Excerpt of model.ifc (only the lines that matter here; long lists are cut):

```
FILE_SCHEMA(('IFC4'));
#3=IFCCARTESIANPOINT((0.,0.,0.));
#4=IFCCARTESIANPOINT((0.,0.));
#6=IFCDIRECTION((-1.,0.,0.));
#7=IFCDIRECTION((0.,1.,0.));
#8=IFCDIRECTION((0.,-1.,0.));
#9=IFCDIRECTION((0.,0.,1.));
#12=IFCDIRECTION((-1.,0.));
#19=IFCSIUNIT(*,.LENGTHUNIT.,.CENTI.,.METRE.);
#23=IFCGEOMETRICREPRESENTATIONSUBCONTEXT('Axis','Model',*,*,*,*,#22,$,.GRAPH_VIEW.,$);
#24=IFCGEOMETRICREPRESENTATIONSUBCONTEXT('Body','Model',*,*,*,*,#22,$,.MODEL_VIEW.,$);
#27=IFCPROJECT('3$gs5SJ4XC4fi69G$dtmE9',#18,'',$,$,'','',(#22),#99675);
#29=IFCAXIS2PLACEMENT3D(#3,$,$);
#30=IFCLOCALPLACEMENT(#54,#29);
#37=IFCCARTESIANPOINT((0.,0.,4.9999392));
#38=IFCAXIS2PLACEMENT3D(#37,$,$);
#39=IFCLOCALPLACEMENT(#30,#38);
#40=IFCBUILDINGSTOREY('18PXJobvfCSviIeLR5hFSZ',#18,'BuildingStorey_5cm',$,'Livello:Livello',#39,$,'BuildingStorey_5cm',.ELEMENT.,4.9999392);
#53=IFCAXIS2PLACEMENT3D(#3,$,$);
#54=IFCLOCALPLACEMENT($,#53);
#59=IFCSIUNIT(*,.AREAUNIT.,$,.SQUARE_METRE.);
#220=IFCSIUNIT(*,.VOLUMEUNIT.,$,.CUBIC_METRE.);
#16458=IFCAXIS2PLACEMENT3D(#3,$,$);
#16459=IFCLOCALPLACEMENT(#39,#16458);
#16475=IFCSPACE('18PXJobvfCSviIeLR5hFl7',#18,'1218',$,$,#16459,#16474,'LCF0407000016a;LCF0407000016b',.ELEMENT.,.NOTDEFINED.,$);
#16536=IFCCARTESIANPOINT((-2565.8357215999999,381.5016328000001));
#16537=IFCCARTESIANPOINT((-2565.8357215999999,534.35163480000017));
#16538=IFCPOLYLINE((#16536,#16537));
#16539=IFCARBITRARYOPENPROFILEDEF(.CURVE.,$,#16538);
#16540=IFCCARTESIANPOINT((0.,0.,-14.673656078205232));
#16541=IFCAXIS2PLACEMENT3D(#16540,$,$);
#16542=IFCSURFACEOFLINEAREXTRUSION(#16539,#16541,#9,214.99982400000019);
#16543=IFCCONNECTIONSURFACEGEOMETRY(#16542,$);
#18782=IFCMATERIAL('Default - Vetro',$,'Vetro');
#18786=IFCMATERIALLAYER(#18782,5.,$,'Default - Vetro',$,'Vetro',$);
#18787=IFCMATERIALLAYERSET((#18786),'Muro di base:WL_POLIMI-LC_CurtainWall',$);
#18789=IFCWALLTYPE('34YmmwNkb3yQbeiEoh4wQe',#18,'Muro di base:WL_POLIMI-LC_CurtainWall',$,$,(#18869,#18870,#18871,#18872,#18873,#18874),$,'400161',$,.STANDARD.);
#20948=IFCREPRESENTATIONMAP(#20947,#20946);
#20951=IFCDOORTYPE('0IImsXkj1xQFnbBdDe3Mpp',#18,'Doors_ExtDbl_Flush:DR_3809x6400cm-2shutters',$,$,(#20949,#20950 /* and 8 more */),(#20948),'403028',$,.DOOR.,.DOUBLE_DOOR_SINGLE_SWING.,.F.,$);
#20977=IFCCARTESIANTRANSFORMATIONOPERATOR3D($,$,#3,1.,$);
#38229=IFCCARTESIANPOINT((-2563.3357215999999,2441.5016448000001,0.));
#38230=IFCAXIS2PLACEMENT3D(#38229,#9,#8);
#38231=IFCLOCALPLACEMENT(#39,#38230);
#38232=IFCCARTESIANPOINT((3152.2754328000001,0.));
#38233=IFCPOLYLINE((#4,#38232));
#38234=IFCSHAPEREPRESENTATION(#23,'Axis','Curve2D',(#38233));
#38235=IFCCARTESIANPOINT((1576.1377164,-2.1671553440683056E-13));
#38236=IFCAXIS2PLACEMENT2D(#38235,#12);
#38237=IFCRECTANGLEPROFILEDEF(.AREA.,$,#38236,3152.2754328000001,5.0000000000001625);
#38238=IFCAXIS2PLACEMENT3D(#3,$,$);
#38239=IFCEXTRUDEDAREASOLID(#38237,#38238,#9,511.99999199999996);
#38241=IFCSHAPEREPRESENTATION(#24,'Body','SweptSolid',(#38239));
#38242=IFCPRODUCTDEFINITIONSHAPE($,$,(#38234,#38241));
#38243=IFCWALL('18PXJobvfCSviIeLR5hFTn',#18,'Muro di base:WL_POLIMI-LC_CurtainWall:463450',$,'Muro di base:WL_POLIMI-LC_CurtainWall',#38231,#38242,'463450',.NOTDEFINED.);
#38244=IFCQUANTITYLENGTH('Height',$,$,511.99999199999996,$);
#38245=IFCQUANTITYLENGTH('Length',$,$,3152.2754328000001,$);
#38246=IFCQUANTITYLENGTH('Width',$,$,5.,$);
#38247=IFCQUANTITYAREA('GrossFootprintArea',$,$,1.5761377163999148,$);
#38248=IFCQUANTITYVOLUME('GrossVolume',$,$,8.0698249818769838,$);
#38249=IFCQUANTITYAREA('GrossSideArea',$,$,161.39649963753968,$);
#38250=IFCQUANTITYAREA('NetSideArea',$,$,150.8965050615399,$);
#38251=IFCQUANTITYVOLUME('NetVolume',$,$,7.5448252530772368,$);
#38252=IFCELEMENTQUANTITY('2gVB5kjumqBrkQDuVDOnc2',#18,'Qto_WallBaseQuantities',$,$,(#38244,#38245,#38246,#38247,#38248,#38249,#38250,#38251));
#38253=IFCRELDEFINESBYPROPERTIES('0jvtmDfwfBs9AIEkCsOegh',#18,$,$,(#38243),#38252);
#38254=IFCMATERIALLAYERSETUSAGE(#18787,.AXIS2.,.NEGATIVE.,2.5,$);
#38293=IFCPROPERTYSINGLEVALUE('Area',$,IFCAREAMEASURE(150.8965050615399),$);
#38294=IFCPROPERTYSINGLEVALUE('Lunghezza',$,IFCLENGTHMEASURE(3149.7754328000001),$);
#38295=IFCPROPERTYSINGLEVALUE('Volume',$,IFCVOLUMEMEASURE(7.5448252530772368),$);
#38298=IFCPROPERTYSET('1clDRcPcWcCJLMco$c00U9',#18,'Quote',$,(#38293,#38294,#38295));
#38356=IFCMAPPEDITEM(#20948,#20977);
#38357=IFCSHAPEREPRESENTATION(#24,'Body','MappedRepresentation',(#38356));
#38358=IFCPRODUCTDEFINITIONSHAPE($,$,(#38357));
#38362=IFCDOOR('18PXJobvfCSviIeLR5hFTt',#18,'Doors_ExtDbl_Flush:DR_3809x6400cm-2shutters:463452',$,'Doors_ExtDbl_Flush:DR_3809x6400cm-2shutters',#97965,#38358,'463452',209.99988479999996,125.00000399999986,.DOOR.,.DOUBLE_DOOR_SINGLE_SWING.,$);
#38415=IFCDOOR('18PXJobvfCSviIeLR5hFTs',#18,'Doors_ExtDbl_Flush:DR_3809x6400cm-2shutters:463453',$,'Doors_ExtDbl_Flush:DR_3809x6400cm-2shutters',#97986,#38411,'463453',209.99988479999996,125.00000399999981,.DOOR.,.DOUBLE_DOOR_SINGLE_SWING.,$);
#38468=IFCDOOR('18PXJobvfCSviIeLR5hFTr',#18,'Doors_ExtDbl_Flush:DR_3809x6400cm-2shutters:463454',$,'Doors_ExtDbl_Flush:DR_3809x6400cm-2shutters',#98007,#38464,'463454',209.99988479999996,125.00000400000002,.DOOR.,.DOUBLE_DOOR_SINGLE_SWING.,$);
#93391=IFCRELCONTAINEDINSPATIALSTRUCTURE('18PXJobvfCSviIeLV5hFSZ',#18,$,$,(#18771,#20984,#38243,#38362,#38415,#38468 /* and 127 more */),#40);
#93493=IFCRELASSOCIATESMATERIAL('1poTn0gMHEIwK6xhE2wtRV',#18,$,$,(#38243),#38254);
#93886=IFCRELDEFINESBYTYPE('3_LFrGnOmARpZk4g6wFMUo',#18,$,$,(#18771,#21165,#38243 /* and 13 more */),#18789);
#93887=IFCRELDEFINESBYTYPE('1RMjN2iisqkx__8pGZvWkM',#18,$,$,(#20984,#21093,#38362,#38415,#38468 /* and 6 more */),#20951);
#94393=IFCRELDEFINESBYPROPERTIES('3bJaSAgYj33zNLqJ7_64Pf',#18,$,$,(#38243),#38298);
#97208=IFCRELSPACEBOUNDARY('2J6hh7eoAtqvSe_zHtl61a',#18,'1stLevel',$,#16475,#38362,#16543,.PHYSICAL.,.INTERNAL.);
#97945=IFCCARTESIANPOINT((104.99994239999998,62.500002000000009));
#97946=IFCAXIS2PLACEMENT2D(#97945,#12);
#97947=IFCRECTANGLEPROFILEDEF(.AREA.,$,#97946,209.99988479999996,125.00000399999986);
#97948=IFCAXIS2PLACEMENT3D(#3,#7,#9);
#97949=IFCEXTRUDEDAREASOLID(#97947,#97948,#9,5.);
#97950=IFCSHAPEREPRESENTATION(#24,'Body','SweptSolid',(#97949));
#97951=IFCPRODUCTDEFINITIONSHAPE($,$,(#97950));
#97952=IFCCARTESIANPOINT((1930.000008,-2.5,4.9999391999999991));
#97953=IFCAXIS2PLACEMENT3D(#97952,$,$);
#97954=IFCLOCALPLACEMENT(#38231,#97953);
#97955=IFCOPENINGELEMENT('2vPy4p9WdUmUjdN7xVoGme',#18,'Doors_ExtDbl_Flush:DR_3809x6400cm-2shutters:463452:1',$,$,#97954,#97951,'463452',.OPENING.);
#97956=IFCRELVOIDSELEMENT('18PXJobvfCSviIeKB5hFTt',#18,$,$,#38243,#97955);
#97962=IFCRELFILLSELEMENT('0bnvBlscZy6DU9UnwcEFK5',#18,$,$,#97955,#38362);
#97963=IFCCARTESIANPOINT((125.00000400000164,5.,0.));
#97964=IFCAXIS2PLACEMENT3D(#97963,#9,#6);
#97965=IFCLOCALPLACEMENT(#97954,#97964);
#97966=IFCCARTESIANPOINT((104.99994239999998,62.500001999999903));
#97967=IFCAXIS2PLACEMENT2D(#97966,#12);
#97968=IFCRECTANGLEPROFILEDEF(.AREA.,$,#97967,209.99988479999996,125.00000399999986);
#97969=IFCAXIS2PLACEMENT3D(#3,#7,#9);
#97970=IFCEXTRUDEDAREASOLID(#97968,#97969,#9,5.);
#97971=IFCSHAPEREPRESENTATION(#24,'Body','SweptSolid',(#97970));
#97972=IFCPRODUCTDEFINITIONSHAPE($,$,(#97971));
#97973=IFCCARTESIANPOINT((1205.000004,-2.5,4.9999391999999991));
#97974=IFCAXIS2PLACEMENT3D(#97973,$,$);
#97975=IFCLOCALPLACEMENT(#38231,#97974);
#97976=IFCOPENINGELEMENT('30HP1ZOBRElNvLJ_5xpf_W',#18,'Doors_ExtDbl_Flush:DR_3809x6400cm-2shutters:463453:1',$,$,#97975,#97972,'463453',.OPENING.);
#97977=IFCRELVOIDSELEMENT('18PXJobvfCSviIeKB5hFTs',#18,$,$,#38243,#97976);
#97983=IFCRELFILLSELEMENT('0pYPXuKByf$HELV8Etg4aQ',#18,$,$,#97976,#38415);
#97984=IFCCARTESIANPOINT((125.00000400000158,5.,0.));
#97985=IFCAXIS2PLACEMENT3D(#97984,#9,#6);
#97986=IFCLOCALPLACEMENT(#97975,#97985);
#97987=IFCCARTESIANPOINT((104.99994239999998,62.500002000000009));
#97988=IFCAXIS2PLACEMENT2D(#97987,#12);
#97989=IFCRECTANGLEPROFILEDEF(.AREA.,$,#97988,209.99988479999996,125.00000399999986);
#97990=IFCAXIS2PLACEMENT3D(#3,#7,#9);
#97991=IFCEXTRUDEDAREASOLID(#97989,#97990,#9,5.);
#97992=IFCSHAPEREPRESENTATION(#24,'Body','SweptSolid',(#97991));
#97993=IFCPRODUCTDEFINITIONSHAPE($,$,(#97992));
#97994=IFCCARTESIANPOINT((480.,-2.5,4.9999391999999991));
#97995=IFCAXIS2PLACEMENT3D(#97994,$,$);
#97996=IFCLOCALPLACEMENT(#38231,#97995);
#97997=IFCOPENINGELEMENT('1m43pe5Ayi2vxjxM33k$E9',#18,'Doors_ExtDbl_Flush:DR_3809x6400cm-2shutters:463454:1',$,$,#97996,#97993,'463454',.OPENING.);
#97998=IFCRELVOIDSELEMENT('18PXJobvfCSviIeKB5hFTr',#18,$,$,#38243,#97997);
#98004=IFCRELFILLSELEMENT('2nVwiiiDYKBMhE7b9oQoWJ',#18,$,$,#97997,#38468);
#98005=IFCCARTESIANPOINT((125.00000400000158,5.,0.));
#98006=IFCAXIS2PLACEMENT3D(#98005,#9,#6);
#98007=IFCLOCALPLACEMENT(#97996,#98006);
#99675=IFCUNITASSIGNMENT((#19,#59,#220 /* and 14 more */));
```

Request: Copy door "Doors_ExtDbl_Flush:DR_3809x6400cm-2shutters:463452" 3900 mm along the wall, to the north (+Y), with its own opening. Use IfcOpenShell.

```python
import numpy as np
import ifcopenshell
import ifcopenshell.api.feature
import ifcopenshell.api.geometry
import ifcopenshell.api.pset
import ifcopenshell.api.root
import ifcopenshell.geom
import ifcopenshell.util.element
import ifcopenshell.util.placement
import ifcopenshell.util.shape
import ifcopenshell.util.unit

model = ifcopenshell.open("model.ifc")
unit_scale = ifcopenshell.util.unit.calculate_unit_scale(model)
area_scale = ifcopenshell.util.unit.calculate_unit_scale(model, "AREAUNIT")
volume_scale = ifcopenshell.util.unit.calculate_unit_scale(model, "VOLUMEUNIT")
settings = ifcopenshell.geom.settings()


def volume(element):
    """Net volume in cubic metres, openings subtracted."""
    shape = ifcopenshell.geom.create_shape(settings, element)
    return ifcopenshell.util.shape.get_volume(shape.geometry)


def reuse_history(source, copy):
    """copy_class also copies each property set's owner history, people and application; keep the originals."""
    for rel in copy.IsDefinedBy:
        if rel.is_a("IfcRelDefinesByProperties") and (history := rel.RelatingPropertyDefinition.OwnerHistory):
            rel.RelatingPropertyDefinition.OwnerHistory = source.OwnerHistory
            ifcopenshell.util.element.remove_deep2(model, history)


door = model.by_guid("18PXJobvfCSviIeLR5hFTt")
opening = door.FillsVoids[0].RelatingOpeningElement
wall = opening.VoidsElements[0].RelatingBuildingElement
before = volume(wall)
shift = ifcopenshell.util.placement.get_local_placement(wall.ObjectPlacement)[:3, 0] * -3.9 / unit_scale

# copy_class copies the void relationship, type, container and properties, but no geometry.
new_opening = ifcopenshell.api.root.copy_class(model, product=opening)
new_opening.Representation = ifcopenshell.util.element.copy_deep(
    model, opening.Representation, exclude=["IfcGeometricRepresentationContext", "IfcRepresentationMap"]
)
new_opening.Name = "Doors_ExtDbl_Flush:DR_3809x6400cm-2shutters"
new_opening.Tag = None
reuse_history(opening, new_opening)
new_door = ifcopenshell.api.root.copy_class(model, product=door)
new_door.Representation = ifcopenshell.util.element.copy_deep(
    model, door.Representation, exclude=["IfcGeometricRepresentationContext", "IfcRepresentationMap"]
)
new_door.Name = "Doors_ExtDbl_Flush:DR_3809x6400cm-2shutters"
new_door.Tag = None
reuse_history(door, new_door)
ifcopenshell.api.feature.add_filling(model, opening=new_opening, element=new_door)

for old, new in ((opening, new_opening), (door, new_door)):
    matrix = ifcopenshell.util.placement.get_local_placement(old.ObjectPlacement)
    matrix[:3, 3] += shift
    ifcopenshell.api.geometry.edit_object_placement(model, product=new, matrix=matrix, is_si=False)

# The copied space boundaries still share their surfaces with the original.
for rel in new_door.ProvidesBoundaries:
    if rel.ConnectionGeometry:
        rel.ConnectionGeometry = ifcopenshell.util.element.copy_deep(model, rel.ConnectionGeometry)

# Space boundary surfaces are stored in each space's coordinates; move them too.
for rel in new_door.ProvidesBoundaries:
    if not rel.ConnectionGeometry:
        continue
    surface = rel.ConnectionGeometry.SurfaceOnRelatingElement
    space_matrix = ifcopenshell.util.placement.get_local_placement(rel.RelatingSpace.ObjectPlacement)
    point = np.array(surface.Position.Location.Coordinates) + space_matrix[:3, :3].T @ shift
    surface.Position = model.createIfcAxis2Placement3D(
        model.createIfcCartesianPoint(point.tolist()), surface.Position.Axis, surface.Position.RefDirection
    )

after = volume(wall)
thickness = 0.05  # wall thickness in metres

# Update the wall's stored quantities.
qto = model.by_id(ifcopenshell.util.element.get_pset(wall, "Qto_WallBaseQuantities", should_inherit=False)["id"])
ifcopenshell.api.pset.edit_qto(model, qto=qto, properties={
    "NetSideArea": after / thickness / area_scale,
    "NetVolume": after / volume_scale,
})
pset = model.by_id(ifcopenshell.util.element.get_pset(wall, "Quote", should_inherit=False)["id"])
ifcopenshell.api.pset.edit_pset(model, pset=pset, properties={
    "Area": model.create_entity("IfcAreaMeasure", after / thickness / area_scale),
    "Volume": model.create_entity("IfcVolumeMeasure", after / volume_scale),
})

print(f"wall volume {before:.3f} -> {after:.3f} m3")

model.write("model_v2.ifc")
```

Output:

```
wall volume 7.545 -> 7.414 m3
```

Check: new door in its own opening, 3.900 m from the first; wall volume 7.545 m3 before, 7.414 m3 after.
